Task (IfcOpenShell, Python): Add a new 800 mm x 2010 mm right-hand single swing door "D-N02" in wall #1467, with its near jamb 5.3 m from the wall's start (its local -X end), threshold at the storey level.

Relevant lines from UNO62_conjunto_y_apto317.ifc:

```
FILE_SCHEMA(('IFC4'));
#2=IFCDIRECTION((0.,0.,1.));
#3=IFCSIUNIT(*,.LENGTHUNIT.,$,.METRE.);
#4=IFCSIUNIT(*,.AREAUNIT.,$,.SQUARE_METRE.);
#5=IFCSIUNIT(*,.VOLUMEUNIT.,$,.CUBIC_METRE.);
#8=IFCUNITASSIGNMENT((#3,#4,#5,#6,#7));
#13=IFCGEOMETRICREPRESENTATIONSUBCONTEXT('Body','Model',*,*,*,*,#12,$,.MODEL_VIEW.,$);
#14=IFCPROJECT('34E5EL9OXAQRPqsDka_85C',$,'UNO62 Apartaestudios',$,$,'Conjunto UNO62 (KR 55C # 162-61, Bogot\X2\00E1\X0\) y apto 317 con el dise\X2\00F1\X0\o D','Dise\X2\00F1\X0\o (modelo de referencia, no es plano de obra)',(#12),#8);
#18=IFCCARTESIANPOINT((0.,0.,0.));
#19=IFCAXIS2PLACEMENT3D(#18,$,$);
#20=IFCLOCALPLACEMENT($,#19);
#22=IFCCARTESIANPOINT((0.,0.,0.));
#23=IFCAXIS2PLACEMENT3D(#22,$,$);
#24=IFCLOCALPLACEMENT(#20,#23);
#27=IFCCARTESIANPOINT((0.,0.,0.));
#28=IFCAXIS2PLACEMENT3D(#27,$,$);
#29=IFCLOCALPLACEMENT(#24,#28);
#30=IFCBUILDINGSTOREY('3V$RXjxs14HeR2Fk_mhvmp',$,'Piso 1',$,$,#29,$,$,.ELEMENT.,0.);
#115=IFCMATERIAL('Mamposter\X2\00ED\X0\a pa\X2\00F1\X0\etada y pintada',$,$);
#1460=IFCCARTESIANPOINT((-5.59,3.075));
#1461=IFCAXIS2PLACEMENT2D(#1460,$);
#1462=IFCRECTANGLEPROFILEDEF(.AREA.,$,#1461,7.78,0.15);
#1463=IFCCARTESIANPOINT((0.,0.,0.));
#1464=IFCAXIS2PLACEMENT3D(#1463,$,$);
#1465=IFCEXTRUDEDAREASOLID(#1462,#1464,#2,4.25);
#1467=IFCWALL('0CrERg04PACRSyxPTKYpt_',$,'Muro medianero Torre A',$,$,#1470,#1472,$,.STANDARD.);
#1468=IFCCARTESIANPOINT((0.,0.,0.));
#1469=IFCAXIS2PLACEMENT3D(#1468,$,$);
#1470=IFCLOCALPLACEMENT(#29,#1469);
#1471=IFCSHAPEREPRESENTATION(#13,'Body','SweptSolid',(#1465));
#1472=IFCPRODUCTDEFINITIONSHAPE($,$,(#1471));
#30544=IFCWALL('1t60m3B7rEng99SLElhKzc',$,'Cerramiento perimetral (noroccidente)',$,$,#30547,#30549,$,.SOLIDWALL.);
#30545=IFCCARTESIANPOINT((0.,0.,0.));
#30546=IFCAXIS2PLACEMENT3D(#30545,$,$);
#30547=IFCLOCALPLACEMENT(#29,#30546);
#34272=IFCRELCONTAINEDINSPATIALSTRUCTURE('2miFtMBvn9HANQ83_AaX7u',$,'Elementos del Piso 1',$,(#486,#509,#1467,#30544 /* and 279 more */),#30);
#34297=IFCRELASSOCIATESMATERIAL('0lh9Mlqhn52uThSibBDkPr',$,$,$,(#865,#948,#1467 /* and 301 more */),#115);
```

```python
import numpy as np
import ifcopenshell
import ifcopenshell.api.feature
import ifcopenshell.api.geometry
import ifcopenshell.api.root
import ifcopenshell.api.spatial
import ifcopenshell.geom
import ifcopenshell.util.element
import ifcopenshell.util.placement
import ifcopenshell.util.representation
import ifcopenshell.util.shape
import ifcopenshell.util.unit

model = ifcopenshell.open("UNO62_conjunto_y_apto317.ifc")
unit_scale = ifcopenshell.util.unit.calculate_unit_scale(model)
settings = ifcopenshell.geom.settings()


def volume(element):
    """Net volume in cubic metres, openings subtracted."""
    shape = ifcopenshell.geom.create_shape(settings, element)
    return ifcopenshell.util.shape.get_volume(shape.geometry)


wall = model.by_guid("0CrERg04PACRSyxPTKYpt_")
storey = ifcopenshell.util.element.get_container(wall, ifc_class="IfcBuildingStorey")
context = ifcopenshell.util.representation.get_context(model, "Model", "Body", "MODEL_VIEW")
before = volume(wall)

width, height, from_end, sill = 0.8, 2.01, 5.3, 0.0  # metres

# The wall runs along its own X axis, and the end named is its -X end.
wall_shape = ifcopenshell.geom.create_shape(settings, wall)
x, y, z = ifcopenshell.util.shape.get_vertices(wall_shape.geometry).T
start = x.min() + from_end
face, thickness = float(y.min()), float(y.max() - y.min())
wall_matrix = ifcopenshell.util.placement.get_local_placement(wall.ObjectPlacement)
level = ifcopenshell.util.placement.get_local_placement(storey.ObjectPlacement)[2, 3]


def in_wall(x, y):
    """Placement at x, y metres in the wall's axes, at sill height."""
    matrix = wall_matrix.copy()
    matrix[:, 3] = wall_matrix @ np.array([x / unit_scale, y / unit_scale, 0.0, 1.0])
    matrix[2, 3] = level + sill / unit_scale
    return matrix


# Opening: a box that overshoots both wall faces by 50 mm.
opening = ifcopenshell.api.root.create_entity(model, ifc_class="IfcOpeningElement", predefined_type="OPENING")
box = ifcopenshell.api.geometry.add_wall_representation(
    model, context=context, length=width, height=height, thickness=thickness + 0.1
)
ifcopenshell.api.geometry.assign_representation(model, product=opening, representation=box)
ifcopenshell.api.geometry.edit_object_placement(model, product=opening, matrix=in_wall(start, face - 0.05), is_si=False)
ifcopenshell.api.feature.add_feature(model, feature=opening, element=wall)

door = ifcopenshell.api.root.create_entity(model, ifc_class="IfcDoor", name="D-N02", predefined_type="DOOR")
door.OverallWidth, door.OverallHeight = width / unit_scale, height / unit_scale
door.OperationType = "SINGLE_SWING_RIGHT"
body = ifcopenshell.api.geometry.add_door_representation(
    model,
    context=context,
    overall_width=door.OverallWidth,
    overall_height=door.OverallHeight,
    operation_type="SINGLE_SWING_RIGHT",
    lining_properties={"LiningDepth": thickness / unit_scale, "ThresholdDepth": thickness / unit_scale},
)
ifcopenshell.api.geometry.assign_representation(model, product=door, representation=body)
ifcopenshell.api.spatial.assign_container(model, products=[door], relating_structure=storey)
ifcopenshell.api.feature.add_filling(model, opening=opening, element=door)

# The lining spans the wall, so the door starts at the wall face.
ifcopenshell.api.geometry.edit_object_placement(model, product=door, matrix=in_wall(start, face), is_si=False)

after = volume(wall)

print(f"wall volume {before:.3f} -> {after:.3f} m3")

model.write("UNO62_conjunto_y_apto317_v2.ifc")
```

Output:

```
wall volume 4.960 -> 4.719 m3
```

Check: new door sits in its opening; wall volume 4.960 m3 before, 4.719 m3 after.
